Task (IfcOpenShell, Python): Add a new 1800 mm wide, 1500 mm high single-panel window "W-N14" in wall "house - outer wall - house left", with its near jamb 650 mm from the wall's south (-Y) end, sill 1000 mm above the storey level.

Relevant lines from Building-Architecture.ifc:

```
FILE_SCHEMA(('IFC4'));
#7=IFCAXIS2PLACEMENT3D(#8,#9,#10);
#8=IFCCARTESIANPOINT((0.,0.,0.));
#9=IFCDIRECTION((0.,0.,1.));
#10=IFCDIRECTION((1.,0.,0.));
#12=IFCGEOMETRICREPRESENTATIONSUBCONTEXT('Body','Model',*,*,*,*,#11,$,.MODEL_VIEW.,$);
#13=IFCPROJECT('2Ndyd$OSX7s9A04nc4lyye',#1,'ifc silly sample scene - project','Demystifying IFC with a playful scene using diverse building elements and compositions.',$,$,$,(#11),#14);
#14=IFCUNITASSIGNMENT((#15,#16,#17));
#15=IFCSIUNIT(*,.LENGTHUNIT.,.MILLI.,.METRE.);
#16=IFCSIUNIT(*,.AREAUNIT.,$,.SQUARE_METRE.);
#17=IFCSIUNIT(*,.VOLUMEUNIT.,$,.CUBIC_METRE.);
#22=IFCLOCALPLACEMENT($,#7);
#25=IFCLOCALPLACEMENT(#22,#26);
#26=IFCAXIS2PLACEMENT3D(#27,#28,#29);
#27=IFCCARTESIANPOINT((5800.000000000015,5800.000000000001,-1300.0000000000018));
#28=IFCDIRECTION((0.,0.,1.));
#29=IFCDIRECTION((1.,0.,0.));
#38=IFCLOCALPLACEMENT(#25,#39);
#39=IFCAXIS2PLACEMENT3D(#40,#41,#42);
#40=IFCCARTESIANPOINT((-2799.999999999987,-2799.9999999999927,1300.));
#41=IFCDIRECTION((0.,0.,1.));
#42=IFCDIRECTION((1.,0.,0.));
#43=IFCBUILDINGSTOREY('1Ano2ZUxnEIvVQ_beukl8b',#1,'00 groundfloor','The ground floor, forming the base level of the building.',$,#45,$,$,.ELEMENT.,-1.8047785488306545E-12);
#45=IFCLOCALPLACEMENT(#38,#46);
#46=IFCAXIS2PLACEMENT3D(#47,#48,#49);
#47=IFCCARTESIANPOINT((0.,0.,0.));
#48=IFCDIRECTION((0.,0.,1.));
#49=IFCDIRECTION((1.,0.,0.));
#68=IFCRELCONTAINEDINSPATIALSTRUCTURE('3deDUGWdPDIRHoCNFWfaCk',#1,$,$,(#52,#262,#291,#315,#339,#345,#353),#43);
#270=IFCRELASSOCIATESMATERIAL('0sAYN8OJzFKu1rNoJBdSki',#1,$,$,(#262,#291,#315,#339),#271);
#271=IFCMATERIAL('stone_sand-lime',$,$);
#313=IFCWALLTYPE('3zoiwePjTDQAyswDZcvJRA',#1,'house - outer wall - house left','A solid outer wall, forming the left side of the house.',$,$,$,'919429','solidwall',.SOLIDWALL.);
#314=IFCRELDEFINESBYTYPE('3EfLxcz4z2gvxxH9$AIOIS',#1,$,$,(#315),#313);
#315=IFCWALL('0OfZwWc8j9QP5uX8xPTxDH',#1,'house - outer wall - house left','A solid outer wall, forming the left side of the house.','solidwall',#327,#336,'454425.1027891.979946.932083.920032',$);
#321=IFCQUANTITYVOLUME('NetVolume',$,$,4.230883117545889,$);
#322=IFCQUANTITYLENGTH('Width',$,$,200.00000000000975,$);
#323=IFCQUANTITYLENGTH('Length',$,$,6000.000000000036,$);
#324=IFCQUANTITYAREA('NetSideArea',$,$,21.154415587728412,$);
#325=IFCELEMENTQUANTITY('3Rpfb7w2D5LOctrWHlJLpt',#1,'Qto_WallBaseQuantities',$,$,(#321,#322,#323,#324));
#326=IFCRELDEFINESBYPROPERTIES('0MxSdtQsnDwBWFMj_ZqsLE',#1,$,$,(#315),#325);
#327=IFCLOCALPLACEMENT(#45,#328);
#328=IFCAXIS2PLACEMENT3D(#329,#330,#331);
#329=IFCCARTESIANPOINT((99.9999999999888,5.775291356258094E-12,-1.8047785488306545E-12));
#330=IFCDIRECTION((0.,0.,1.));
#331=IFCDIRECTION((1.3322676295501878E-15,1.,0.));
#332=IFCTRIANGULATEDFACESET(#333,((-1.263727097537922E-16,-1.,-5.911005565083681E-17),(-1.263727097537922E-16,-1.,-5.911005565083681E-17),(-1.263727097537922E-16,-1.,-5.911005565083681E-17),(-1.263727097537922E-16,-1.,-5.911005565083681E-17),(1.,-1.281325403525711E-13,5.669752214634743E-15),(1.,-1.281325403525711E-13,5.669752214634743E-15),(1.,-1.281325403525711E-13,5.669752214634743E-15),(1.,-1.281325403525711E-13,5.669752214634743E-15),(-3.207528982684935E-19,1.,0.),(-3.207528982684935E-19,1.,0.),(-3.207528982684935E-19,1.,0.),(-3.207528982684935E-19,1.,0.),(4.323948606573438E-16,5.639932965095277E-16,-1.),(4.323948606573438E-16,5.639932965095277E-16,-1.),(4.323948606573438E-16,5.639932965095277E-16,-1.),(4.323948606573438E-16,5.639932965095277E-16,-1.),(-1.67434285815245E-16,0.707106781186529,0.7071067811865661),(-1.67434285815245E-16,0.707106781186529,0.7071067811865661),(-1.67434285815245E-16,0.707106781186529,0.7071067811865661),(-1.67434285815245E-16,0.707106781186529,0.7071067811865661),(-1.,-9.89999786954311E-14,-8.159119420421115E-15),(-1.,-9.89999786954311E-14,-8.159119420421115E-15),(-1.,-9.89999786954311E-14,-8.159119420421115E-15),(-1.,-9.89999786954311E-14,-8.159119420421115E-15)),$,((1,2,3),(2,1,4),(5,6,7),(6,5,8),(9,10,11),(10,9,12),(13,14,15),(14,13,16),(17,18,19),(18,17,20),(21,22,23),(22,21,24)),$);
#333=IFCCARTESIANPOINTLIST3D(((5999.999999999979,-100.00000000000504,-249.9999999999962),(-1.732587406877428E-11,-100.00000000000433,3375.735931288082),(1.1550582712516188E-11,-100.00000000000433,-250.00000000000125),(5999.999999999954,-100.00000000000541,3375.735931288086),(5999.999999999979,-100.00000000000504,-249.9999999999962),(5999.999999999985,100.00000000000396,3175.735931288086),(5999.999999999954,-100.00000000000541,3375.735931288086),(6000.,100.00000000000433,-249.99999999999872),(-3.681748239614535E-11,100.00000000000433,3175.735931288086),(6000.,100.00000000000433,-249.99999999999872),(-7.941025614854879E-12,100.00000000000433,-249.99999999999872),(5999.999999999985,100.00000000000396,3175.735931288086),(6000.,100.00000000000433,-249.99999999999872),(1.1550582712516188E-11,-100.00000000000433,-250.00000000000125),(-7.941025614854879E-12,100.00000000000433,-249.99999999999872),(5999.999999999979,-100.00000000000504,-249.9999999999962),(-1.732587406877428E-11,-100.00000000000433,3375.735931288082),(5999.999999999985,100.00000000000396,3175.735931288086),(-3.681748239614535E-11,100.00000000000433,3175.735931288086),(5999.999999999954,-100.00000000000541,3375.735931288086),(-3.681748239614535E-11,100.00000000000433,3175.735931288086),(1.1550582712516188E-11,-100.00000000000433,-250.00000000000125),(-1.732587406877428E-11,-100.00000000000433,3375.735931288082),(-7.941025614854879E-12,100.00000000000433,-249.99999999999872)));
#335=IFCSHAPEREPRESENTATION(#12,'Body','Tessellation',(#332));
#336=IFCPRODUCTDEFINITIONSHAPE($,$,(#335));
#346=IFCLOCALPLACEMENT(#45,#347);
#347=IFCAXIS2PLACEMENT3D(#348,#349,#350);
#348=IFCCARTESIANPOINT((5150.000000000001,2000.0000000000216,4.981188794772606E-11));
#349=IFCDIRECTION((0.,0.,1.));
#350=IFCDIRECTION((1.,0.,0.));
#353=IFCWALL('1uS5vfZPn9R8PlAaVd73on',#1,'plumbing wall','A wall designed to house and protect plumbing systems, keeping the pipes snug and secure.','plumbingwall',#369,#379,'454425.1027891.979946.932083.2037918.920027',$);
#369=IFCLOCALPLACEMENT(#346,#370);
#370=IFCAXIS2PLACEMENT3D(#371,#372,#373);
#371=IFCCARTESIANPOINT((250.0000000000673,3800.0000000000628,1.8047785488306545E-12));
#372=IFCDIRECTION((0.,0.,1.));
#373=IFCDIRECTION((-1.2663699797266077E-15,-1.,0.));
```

```python
import numpy as np
import ifcopenshell
import ifcopenshell.api.feature
import ifcopenshell.api.geometry
import ifcopenshell.api.pset
import ifcopenshell.api.root
import ifcopenshell.api.spatial
import ifcopenshell.geom
import ifcopenshell.util.element
import ifcopenshell.util.placement
import ifcopenshell.util.representation
import ifcopenshell.util.shape
import ifcopenshell.util.unit

model = ifcopenshell.open("Building-Architecture.ifc")
unit_scale = ifcopenshell.util.unit.calculate_unit_scale(model)
area_scale = ifcopenshell.util.unit.calculate_unit_scale(model, "AREAUNIT")
volume_scale = ifcopenshell.util.unit.calculate_unit_scale(model, "VOLUMEUNIT")
settings = ifcopenshell.geom.settings()


def volume(element):
    """Net volume in cubic metres, openings subtracted."""
    shape = ifcopenshell.geom.create_shape(settings, element)
    return ifcopenshell.util.shape.get_volume(shape.geometry)


wall = model.by_guid("0OfZwWc8j9QP5uX8xPTxDH")
storey = ifcopenshell.util.element.get_container(wall, ifc_class="IfcBuildingStorey")
context = ifcopenshell.util.representation.get_context(model, "Model", "Body", "MODEL_VIEW")
before = volume(wall)

width, height, from_end, sill = 1.8, 1.5, 0.65, 1  # metres

# The wall runs along its own X axis, and the end named is its -X end.
wall_shape = ifcopenshell.geom.create_shape(settings, wall)
x, y, z = ifcopenshell.util.shape.get_vertices(wall_shape.geometry).T
start = x.min() + from_end
face, thickness = float(y.min()), float(y.max() - y.min())
wall_matrix = ifcopenshell.util.placement.get_local_placement(wall.ObjectPlacement)
level = ifcopenshell.util.placement.get_local_placement(storey.ObjectPlacement)[2, 3]


def in_wall(x, y):
    """Placement at x, y metres in the wall's axes, at sill height."""
    matrix = wall_matrix.copy()
    matrix[:, 3] = wall_matrix @ np.array([x / unit_scale, y / unit_scale, 0.0, 1.0])
    matrix[2, 3] = level + sill / unit_scale
    return matrix


# Opening: a box that overshoots both wall faces by 50 mm.
opening = ifcopenshell.api.root.create_entity(model, ifc_class="IfcOpeningElement", predefined_type="OPENING")
box = ifcopenshell.api.geometry.add_wall_representation(
    model, context=context, length=width, height=height, thickness=thickness + 0.1
)
ifcopenshell.api.geometry.assign_representation(model, product=opening, representation=box)
ifcopenshell.api.geometry.edit_object_placement(model, product=opening, matrix=in_wall(start, face - 0.05), is_si=False)
ifcopenshell.api.feature.add_feature(model, feature=opening, element=wall)

window = ifcopenshell.api.root.create_entity(model, ifc_class="IfcWindow", name="W-N14", predefined_type="WINDOW")
window.OverallWidth, window.OverallHeight = width / unit_scale, height / unit_scale
window.PartitioningType = "SINGLE_PANEL"
body = ifcopenshell.api.geometry.add_window_representation(
    model,
    context=context,
    overall_width=window.OverallWidth,
    overall_height=window.OverallHeight,
    partition_type="SINGLE_PANEL",
)
ifcopenshell.api.geometry.assign_representation(model, product=window, representation=body)
ifcopenshell.api.spatial.assign_container(model, products=[window], relating_structure=storey)
ifcopenshell.api.feature.add_filling(model, opening=opening, element=window)

# Centre the window in the wall's thickness.
ifcopenshell.api.geometry.edit_object_placement(model, product=window, matrix=in_wall(start, face), is_si=False)
window_shape = ifcopenshell.geom.create_shape(settings, window)
depth = ifcopenshell.util.shape.get_vertices(window_shape.geometry)[:, 1]
offset = face + thickness / 2 - (depth.min() + depth.max()) / 2
ifcopenshell.api.geometry.edit_object_placement(model, product=window, matrix=in_wall(start, offset), is_si=False)

after = volume(wall)

# Update the wall's stored quantities.
qto = model.by_id(ifcopenshell.util.element.get_pset(wall, "Qto_WallBaseQuantities", should_inherit=False)["id"])
ifcopenshell.api.pset.edit_qto(model, qto=qto, properties={
    "NetVolume": after / volume_scale,
    "NetSideArea": after / thickness / area_scale,
})

print(f"wall volume {before:.3f} -> {after:.3f} m3")

model.write("Building-Architecture_v2.ifc")
```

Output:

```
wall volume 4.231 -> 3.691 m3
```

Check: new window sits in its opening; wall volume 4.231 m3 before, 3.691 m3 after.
